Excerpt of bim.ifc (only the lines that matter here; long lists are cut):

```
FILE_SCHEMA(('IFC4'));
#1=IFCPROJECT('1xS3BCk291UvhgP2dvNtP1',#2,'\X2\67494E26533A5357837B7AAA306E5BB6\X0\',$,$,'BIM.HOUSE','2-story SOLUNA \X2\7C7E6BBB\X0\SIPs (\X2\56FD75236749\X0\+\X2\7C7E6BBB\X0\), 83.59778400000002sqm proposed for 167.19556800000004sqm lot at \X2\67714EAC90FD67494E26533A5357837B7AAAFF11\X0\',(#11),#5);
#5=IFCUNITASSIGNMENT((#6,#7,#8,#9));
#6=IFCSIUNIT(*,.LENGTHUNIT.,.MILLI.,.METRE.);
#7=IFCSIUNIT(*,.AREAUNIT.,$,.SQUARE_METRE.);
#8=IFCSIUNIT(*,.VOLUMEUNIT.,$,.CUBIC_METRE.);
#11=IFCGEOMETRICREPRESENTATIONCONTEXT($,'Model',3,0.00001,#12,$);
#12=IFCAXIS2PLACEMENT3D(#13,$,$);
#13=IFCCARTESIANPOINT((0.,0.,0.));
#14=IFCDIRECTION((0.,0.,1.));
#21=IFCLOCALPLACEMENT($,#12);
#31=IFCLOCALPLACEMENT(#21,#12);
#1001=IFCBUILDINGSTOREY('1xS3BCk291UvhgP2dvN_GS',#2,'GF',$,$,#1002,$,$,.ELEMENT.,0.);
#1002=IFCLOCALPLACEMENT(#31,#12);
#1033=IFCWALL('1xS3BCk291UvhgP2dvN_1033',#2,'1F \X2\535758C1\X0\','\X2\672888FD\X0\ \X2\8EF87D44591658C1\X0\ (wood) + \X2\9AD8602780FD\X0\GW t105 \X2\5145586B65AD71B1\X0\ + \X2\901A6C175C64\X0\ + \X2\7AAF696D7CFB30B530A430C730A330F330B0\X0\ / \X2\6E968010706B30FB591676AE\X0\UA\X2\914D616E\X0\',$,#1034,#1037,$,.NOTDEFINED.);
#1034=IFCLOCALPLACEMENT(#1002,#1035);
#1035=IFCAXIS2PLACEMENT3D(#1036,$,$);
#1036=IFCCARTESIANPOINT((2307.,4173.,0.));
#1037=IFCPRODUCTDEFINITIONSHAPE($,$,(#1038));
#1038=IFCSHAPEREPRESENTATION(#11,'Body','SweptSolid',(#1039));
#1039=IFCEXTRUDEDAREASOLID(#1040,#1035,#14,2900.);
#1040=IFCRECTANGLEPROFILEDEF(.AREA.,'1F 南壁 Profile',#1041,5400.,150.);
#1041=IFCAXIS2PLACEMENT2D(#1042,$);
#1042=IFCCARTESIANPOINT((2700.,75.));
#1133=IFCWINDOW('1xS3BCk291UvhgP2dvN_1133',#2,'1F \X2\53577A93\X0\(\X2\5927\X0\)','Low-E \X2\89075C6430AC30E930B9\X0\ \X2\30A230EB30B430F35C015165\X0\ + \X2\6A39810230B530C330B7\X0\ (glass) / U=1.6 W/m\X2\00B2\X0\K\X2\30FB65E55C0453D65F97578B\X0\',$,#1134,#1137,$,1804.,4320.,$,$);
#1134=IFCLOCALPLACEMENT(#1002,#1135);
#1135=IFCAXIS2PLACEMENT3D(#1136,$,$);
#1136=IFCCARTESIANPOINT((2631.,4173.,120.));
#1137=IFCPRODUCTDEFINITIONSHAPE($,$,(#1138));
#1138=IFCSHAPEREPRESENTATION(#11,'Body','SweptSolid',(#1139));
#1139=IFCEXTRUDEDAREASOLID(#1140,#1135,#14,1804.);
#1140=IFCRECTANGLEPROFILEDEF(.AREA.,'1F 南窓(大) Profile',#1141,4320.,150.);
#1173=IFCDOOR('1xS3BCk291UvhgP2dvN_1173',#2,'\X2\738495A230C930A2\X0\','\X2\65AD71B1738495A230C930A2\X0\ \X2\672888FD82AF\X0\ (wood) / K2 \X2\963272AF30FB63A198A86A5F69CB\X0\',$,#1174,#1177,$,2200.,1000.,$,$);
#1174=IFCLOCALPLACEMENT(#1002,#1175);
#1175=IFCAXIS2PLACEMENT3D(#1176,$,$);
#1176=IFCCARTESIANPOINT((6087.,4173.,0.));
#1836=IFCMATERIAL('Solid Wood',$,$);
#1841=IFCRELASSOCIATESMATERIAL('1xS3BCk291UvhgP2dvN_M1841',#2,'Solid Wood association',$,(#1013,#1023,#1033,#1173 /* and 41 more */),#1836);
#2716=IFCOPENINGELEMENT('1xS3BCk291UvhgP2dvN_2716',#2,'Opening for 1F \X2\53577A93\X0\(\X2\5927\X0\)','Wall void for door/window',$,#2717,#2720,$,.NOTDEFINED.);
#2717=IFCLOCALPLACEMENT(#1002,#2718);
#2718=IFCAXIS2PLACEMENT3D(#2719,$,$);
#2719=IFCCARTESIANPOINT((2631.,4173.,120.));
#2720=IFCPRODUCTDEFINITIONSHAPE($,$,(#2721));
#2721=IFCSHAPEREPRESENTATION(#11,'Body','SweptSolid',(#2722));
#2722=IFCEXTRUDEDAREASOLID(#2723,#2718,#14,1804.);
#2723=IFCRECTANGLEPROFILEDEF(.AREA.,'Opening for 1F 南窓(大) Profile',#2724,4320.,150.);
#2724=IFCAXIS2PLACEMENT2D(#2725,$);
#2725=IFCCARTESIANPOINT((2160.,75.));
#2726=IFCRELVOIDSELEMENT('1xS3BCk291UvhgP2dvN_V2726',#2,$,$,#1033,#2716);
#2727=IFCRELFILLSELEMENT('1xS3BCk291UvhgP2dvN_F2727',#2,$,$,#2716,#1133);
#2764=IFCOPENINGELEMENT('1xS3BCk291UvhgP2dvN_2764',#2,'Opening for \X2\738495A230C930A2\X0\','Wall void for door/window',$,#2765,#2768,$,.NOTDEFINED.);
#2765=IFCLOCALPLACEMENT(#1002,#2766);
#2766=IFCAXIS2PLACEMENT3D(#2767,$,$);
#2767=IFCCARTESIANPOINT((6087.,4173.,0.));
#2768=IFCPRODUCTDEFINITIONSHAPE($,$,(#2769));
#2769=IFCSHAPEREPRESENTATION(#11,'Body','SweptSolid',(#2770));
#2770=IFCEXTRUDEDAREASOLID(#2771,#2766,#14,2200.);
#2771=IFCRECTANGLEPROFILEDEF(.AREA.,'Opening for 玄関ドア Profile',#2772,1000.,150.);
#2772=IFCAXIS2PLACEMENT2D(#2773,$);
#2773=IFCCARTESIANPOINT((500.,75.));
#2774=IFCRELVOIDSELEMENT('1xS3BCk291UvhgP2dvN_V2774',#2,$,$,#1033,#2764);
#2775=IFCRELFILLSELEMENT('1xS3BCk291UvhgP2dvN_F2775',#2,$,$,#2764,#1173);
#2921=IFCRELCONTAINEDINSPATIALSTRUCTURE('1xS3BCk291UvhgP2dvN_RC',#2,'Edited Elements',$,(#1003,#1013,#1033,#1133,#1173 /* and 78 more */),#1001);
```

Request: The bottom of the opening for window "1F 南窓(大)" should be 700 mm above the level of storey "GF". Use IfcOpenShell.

```python
import numpy as np
import ifcopenshell
import ifcopenshell.api.geometry
import ifcopenshell.geom
import ifcopenshell.util.element
import ifcopenshell.util.placement
import ifcopenshell.util.shape
import ifcopenshell.util.unit

model = ifcopenshell.open("bim.ifc")
unit_scale = ifcopenshell.util.unit.calculate_unit_scale(model)

window = model.by_guid("1xS3BCk291UvhgP2dvN_1133")
opening = window.FillsVoids[0].RelatingOpeningElement
storey = ifcopenshell.util.element.get_container(window, ifc_class="IfcBuildingStorey")
level = ifcopenshell.util.placement.get_local_placement(storey.ObjectPlacement)[2, 3]

# The opening's origin need not be at the sill, so measure its lowest point.
shape = ifcopenshell.geom.create_shape(ifcopenshell.geom.settings(), opening)
bottom = ifcopenshell.util.shape.get_shape_bottom_elevation(shape, shape.geometry) / unit_scale
dz = level + 0.7 / unit_scale - bottom

shift = np.array([0.0, 0.0, dz])
# The window is not placed relative to its opening, so move both.
for product in (opening, window):
    matrix = ifcopenshell.util.placement.get_local_placement(product.ObjectPlacement)
    matrix[:3, 3] += shift
    ifcopenshell.api.geometry.edit_object_placement(model, product=product, matrix=matrix, is_si=False)

print(f"moved by {dz * unit_scale:+.3f} m")

model.write("bim_rev.ifc")
```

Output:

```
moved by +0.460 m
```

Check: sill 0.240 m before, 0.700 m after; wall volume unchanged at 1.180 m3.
